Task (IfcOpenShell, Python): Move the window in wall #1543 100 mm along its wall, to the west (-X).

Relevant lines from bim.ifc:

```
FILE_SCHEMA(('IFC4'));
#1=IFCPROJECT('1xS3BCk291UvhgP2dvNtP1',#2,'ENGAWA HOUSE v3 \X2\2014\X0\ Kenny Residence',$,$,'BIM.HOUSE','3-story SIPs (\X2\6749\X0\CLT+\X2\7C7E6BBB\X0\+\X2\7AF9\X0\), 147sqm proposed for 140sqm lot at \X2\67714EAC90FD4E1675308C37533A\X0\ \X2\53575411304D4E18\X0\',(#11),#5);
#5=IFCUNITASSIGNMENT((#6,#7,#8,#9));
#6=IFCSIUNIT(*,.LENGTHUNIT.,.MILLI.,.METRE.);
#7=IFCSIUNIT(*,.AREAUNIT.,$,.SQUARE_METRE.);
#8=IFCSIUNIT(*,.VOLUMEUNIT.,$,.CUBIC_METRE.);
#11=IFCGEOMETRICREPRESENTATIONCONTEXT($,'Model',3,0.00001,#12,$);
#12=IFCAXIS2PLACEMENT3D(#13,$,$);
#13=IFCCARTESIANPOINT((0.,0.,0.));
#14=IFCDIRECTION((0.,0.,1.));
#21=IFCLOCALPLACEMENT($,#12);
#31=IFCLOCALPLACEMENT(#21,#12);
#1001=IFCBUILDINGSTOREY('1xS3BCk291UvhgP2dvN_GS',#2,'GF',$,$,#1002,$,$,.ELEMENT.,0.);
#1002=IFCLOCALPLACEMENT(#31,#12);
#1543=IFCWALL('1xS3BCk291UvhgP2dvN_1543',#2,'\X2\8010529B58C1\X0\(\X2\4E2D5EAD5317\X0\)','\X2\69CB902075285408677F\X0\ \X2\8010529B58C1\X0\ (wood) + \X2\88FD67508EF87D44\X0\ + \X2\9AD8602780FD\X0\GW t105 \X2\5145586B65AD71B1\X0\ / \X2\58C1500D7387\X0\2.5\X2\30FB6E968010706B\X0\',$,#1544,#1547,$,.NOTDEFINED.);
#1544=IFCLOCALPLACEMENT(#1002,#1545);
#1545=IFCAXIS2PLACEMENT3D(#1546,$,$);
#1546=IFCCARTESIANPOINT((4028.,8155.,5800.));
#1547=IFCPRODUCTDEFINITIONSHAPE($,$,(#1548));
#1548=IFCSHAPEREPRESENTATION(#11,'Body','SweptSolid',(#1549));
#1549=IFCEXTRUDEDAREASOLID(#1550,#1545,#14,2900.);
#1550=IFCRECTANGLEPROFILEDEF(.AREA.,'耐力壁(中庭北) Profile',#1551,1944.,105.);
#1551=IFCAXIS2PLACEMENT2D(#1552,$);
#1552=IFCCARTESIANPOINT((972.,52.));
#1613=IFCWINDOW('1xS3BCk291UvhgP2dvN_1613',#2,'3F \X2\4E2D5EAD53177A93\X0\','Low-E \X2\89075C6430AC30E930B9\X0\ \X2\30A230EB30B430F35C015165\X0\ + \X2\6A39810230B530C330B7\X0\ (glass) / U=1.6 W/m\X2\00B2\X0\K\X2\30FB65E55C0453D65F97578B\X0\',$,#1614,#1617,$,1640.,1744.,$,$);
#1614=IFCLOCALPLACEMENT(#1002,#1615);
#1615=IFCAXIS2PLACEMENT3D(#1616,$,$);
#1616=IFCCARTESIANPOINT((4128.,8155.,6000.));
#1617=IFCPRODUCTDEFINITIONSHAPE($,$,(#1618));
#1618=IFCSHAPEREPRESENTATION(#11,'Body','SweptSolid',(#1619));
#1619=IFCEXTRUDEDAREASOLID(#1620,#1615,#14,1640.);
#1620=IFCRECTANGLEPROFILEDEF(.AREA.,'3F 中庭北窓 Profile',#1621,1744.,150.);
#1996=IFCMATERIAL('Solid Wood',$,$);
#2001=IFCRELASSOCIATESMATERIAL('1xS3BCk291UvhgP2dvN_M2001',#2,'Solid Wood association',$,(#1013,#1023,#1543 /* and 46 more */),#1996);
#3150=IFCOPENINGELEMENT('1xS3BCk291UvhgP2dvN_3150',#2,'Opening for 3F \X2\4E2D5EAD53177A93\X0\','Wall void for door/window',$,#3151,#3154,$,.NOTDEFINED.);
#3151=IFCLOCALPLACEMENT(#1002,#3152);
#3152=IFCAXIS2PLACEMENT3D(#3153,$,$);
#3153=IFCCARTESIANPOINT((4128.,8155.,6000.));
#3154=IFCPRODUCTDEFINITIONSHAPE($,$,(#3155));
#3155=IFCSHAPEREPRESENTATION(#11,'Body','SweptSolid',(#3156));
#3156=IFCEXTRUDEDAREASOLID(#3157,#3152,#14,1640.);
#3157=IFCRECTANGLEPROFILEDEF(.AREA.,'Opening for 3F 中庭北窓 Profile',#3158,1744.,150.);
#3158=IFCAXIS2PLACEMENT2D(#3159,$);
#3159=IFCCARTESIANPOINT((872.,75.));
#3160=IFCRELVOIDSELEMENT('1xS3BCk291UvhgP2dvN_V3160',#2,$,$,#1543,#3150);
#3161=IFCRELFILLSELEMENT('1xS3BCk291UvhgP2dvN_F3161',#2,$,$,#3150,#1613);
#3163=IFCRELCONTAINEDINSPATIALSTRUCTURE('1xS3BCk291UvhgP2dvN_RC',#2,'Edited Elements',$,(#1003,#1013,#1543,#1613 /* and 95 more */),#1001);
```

```python
import ifcopenshell
import ifcopenshell.api.geometry
import ifcopenshell.util.placement
import ifcopenshell.util.unit

model = ifcopenshell.open("bim.ifc")
unit_scale = ifcopenshell.util.unit.calculate_unit_scale(model)

window = model.by_guid("1xS3BCk291UvhgP2dvN_1613")
opening = window.FillsVoids[0].RelatingOpeningElement
wall = opening.VoidsElements[0].RelatingBuildingElement

wall_matrix = ifcopenshell.util.placement.get_local_placement(wall.ObjectPlacement)
shift = wall_matrix[:3, 0] * -0.1 / unit_scale
before = ifcopenshell.util.placement.get_local_placement(window.ObjectPlacement)[:3, 3].copy()

# The window is not placed relative to its opening, so move both.
for product in (opening, window):
    matrix = ifcopenshell.util.placement.get_local_placement(product.ObjectPlacement)
    matrix[:3, 3] += shift
    ifcopenshell.api.geometry.edit_object_placement(model, product=product, matrix=matrix, is_si=False)

after = ifcopenshell.util.placement.get_local_placement(window.ObjectPlacement)[:3, 3]
print("window moved by", (after - before).round(3) + 0.0)

model.write("bim_v2.ifc")
```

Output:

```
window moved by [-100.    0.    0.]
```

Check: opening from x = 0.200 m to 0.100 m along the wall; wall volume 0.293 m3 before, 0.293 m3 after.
